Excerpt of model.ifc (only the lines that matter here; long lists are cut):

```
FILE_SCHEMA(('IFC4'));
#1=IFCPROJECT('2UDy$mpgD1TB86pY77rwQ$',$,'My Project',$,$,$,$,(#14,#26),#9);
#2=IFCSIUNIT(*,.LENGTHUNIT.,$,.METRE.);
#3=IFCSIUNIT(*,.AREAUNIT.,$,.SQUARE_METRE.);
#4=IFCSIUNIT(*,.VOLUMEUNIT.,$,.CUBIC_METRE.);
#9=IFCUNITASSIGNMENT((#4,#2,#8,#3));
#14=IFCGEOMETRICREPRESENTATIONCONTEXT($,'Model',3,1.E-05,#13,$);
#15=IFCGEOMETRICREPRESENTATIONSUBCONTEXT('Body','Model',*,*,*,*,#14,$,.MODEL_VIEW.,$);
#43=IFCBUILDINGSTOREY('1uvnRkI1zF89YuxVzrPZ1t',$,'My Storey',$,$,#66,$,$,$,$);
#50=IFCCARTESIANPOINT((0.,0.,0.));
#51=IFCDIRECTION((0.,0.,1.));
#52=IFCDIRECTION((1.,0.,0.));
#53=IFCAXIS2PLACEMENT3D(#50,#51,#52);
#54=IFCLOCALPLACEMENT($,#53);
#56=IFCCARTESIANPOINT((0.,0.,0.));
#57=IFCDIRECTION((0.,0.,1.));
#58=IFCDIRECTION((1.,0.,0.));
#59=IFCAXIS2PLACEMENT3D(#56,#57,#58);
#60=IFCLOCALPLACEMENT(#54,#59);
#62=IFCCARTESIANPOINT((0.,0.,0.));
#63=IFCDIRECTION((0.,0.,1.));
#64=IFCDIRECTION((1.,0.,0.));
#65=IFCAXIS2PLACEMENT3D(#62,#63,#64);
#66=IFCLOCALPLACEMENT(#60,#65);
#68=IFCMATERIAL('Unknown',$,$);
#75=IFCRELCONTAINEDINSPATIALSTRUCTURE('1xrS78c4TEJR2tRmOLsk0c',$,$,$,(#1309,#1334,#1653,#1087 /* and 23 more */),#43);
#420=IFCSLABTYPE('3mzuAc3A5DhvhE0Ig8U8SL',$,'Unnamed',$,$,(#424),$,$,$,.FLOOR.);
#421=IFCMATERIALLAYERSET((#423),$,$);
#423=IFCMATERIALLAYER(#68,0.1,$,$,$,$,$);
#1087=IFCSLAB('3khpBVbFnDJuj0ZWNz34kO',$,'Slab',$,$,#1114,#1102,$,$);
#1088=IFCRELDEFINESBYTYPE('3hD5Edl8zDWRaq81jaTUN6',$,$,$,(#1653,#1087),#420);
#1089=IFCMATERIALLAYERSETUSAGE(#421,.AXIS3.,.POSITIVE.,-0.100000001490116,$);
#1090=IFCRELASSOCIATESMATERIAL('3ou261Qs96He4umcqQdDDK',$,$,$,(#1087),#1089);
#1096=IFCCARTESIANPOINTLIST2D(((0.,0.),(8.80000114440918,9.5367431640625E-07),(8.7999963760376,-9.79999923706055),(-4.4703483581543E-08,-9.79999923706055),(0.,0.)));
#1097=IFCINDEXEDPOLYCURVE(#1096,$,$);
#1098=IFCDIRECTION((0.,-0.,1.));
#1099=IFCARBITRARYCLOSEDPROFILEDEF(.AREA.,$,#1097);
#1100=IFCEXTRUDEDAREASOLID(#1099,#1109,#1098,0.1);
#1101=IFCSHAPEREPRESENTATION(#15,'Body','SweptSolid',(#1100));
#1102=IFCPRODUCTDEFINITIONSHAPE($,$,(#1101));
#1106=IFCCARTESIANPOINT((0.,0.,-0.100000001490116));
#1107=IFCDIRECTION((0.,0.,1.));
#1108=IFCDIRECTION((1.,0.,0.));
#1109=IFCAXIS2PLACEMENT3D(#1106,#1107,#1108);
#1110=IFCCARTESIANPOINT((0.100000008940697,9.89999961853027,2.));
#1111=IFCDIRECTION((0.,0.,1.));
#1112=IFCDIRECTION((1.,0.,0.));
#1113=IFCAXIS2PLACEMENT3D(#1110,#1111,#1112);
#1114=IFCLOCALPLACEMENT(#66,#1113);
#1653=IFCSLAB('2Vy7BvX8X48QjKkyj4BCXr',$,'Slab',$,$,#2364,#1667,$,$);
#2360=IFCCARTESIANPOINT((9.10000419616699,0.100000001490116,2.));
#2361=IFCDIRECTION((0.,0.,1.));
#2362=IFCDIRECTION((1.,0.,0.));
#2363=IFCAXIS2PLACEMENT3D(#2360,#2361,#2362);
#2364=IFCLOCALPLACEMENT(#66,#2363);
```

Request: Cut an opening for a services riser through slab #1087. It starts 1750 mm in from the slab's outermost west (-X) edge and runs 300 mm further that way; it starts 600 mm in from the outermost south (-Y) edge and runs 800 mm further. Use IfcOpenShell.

```python
import numpy as np
import ifcopenshell
import ifcopenshell.api.feature
import ifcopenshell.api.geometry
import ifcopenshell.api.root
import ifcopenshell.geom
import ifcopenshell.util.placement
import ifcopenshell.util.representation
import ifcopenshell.util.shape
import ifcopenshell.util.unit

model = ifcopenshell.open("model.ifc")
unit_scale = ifcopenshell.util.unit.calculate_unit_scale(model)
settings = ifcopenshell.geom.settings()


def volume(element):
    """Net volume in cubic metres, openings subtracted."""
    shape = ifcopenshell.geom.create_shape(settings, element)
    return ifcopenshell.util.shape.get_volume(shape.geometry)


slab = model.by_id(1087)
before = volume(slab)

# Extent in the slab's own axes, in metres. The edges named are its -X and -Y sides.
slab_shape = ifcopenshell.geom.create_shape(settings, slab)
vertices = ifcopenshell.util.shape.get_vertices(slab_shape.geometry)
x_min, y_min, bottom = vertices.min(axis=0)
top = vertices[:, 2].max()

opening = ifcopenshell.api.root.create_entity(model, ifc_class="IfcOpeningElement", name="Services riser opening", predefined_type="OPENING")
context = ifcopenshell.util.representation.get_context(model, "Model", "Body", "MODEL_VIEW")
width, depth = 0.3, 0.8
outline = [(0.0, 0.0), (width, 0.0), (width, depth), (0.0, depth), (0.0, 0.0)]
# Overshoot both faces by 50 mm so the cut is clean.
shape = ifcopenshell.api.geometry.add_slab_representation(
    model, context=context, depth=top - bottom + 0.1, polyline=outline
)
ifcopenshell.api.geometry.assign_representation(model, product=opening, representation=shape)

matrix = ifcopenshell.util.placement.get_local_placement(slab.ObjectPlacement)
matrix[:, 3] = matrix @ np.append(np.array([x_min + 1.75, y_min + 0.6, bottom - 0.05]) / unit_scale, 1.0)
ifcopenshell.api.geometry.edit_object_placement(model, product=opening, matrix=matrix, is_si=False)
ifcopenshell.api.feature.add_feature(model, feature=opening, element=slab)

after = volume(slab)

print(f"slab volume {before:.3f} -> {after:.3f} m3")

model.write("model_rev.ifc")
```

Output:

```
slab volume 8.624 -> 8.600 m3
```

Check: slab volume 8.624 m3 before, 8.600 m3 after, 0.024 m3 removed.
